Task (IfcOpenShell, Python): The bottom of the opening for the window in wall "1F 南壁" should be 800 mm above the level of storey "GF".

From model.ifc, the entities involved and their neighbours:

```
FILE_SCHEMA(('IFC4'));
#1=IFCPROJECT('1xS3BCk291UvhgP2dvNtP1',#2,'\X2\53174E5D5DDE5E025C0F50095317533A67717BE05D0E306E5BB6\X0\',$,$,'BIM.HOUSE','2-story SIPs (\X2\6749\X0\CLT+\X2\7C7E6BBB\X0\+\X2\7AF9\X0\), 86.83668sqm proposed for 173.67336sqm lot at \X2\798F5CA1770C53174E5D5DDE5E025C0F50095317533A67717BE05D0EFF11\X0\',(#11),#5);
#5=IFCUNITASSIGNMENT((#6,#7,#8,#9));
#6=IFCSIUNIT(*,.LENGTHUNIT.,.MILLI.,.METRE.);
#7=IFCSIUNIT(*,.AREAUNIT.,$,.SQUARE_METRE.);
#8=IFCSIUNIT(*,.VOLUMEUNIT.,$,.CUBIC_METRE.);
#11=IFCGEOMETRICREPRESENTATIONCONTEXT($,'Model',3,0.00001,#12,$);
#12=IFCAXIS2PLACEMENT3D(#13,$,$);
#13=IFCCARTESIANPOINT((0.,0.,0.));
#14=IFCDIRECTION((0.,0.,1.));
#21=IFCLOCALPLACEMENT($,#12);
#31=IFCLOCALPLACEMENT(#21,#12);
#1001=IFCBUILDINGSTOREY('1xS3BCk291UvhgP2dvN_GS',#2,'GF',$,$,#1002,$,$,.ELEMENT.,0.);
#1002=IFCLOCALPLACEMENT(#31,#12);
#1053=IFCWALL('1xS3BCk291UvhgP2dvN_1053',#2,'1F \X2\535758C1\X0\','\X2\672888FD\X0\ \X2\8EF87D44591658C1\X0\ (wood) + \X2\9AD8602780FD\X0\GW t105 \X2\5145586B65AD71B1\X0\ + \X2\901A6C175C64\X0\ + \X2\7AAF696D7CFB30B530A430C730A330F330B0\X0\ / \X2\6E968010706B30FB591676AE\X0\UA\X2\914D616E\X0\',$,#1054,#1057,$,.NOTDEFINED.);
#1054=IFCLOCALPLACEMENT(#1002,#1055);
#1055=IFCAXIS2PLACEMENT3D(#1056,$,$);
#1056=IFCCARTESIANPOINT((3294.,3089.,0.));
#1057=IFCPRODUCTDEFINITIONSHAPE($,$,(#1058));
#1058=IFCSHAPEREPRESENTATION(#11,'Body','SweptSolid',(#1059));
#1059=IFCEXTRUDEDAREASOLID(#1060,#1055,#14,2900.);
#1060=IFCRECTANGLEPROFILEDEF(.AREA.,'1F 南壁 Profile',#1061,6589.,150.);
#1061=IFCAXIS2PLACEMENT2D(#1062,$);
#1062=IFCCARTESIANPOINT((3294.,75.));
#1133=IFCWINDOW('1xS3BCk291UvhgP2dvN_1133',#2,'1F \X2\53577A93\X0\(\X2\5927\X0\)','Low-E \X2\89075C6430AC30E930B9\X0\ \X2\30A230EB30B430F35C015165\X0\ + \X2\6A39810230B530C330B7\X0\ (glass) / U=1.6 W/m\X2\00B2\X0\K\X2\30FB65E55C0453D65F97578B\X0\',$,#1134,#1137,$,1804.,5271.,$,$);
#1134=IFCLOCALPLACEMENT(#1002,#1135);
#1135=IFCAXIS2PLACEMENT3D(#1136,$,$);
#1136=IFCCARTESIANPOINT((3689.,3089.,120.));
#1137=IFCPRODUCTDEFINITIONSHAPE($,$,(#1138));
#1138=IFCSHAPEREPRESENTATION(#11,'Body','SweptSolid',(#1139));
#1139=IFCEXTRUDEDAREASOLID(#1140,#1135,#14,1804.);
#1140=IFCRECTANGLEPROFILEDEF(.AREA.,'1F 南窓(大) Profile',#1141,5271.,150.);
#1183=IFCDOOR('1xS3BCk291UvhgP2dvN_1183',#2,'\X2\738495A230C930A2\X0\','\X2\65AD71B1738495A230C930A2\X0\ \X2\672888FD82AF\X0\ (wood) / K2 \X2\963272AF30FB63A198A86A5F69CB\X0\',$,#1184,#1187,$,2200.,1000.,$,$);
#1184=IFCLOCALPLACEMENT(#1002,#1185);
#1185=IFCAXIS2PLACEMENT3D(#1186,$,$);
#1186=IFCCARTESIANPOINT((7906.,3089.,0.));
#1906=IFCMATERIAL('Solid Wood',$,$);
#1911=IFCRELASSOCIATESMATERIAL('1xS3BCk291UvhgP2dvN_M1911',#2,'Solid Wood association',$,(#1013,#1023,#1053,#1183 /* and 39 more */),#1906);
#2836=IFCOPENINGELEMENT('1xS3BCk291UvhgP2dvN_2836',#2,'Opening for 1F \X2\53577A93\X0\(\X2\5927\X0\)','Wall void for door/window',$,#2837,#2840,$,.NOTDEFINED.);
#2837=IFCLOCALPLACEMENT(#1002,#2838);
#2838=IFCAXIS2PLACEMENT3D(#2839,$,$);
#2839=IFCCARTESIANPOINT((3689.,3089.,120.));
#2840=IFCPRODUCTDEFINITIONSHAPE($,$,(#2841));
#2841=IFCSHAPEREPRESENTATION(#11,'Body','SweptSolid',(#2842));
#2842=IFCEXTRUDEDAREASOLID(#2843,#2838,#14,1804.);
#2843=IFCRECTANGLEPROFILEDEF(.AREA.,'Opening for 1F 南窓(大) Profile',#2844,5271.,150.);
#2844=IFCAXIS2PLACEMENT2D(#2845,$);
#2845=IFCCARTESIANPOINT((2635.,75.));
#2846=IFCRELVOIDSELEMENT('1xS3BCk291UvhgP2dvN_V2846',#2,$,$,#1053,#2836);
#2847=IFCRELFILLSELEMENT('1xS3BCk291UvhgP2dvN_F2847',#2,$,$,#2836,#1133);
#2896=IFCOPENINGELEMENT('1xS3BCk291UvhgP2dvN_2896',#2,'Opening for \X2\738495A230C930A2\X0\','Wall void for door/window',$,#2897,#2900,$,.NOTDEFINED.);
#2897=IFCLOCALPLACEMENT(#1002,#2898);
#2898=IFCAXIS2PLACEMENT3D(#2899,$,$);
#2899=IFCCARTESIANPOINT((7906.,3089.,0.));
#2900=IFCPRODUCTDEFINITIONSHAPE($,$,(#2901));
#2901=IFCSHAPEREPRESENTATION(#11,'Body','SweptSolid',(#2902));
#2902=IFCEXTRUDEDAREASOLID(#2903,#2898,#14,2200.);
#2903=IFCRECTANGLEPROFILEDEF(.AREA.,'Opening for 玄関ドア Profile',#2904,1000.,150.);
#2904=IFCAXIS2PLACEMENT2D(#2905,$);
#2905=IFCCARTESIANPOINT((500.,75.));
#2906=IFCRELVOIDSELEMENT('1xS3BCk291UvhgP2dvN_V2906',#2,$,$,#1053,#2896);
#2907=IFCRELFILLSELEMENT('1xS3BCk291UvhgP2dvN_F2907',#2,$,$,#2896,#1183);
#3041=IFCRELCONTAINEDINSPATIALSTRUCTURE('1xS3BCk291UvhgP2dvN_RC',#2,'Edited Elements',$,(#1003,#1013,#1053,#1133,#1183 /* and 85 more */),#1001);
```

```python
import numpy as np
import ifcopenshell
import ifcopenshell.api.geometry
import ifcopenshell.geom
import ifcopenshell.util.element
import ifcopenshell.util.placement
import ifcopenshell.util.shape
import ifcopenshell.util.unit

model = ifcopenshell.open("model.ifc")
unit_scale = ifcopenshell.util.unit.calculate_unit_scale(model)

window = model.by_guid("1xS3BCk291UvhgP2dvN_1133")
opening = window.FillsVoids[0].RelatingOpeningElement
storey = ifcopenshell.util.element.get_container(window, ifc_class="IfcBuildingStorey")
level = ifcopenshell.util.placement.get_local_placement(storey.ObjectPlacement)[2, 3]

# The opening's origin need not be at the sill, so measure its lowest point.
shape = ifcopenshell.geom.create_shape(ifcopenshell.geom.settings(), opening)
bottom = ifcopenshell.util.shape.get_shape_bottom_elevation(shape, shape.geometry) / unit_scale
dz = level + 800.0 - bottom

shift = np.array([0.0, 0.0, dz])
# The window is not placed relative to its opening, so move both.
for product in (opening, window):
    matrix = ifcopenshell.util.placement.get_local_placement(product.ObjectPlacement)
    matrix[:3, 3] += shift
    ifcopenshell.api.geometry.edit_object_placement(model, product=product, matrix=matrix, is_si=False)

print(f"moved by {dz * unit_scale:+.3f} m")

model.write("model_updated.ifc")
```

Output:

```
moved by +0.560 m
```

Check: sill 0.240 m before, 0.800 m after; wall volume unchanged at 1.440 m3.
